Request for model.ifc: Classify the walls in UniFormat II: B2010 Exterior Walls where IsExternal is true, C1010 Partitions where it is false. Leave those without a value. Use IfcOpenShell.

First a look at what the model holds.

```python
import ifcopenshell
import ifcopenshell.util.element

model = ifcopenshell.open("model.ifc")
print(model.schema)
print("classifications:", [c.Name for c in model.by_type("IfcClassification")])
values = [ifcopenshell.util.element.get_pset(e, "Pset_WallCommon", "IsExternal") for e in model.by_type("IfcWall")]
for value in (True, False, None):
    print("IsExternal", value, values.count(value))
```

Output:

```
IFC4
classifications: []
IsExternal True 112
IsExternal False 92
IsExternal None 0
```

```python
import ifcopenshell
import ifcopenshell.api.classification
import ifcopenshell.util.element

model = ifcopenshell.open("model.ifc")

system = ifcopenshell.api.classification.add_classification(model, classification="UniFormat II")

walls = model.by_type("IfcWall")
external = {e: ifcopenshell.util.element.get_pset(e, "Pset_WallCommon", "IsExternal") for e in walls}
for flag, code, name in ((True, "B2010", "Exterior Walls"), (False, "C1010", "Partitions")):
    products = [e for e in walls if external[e] is flag]
    ifcopenshell.api.classification.add_reference(
        model, products=products, classification=system, identification=code, name=name
    )
    print(code, len(products))

model.write("model-out.ifc")
```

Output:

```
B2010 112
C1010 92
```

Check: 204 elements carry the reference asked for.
